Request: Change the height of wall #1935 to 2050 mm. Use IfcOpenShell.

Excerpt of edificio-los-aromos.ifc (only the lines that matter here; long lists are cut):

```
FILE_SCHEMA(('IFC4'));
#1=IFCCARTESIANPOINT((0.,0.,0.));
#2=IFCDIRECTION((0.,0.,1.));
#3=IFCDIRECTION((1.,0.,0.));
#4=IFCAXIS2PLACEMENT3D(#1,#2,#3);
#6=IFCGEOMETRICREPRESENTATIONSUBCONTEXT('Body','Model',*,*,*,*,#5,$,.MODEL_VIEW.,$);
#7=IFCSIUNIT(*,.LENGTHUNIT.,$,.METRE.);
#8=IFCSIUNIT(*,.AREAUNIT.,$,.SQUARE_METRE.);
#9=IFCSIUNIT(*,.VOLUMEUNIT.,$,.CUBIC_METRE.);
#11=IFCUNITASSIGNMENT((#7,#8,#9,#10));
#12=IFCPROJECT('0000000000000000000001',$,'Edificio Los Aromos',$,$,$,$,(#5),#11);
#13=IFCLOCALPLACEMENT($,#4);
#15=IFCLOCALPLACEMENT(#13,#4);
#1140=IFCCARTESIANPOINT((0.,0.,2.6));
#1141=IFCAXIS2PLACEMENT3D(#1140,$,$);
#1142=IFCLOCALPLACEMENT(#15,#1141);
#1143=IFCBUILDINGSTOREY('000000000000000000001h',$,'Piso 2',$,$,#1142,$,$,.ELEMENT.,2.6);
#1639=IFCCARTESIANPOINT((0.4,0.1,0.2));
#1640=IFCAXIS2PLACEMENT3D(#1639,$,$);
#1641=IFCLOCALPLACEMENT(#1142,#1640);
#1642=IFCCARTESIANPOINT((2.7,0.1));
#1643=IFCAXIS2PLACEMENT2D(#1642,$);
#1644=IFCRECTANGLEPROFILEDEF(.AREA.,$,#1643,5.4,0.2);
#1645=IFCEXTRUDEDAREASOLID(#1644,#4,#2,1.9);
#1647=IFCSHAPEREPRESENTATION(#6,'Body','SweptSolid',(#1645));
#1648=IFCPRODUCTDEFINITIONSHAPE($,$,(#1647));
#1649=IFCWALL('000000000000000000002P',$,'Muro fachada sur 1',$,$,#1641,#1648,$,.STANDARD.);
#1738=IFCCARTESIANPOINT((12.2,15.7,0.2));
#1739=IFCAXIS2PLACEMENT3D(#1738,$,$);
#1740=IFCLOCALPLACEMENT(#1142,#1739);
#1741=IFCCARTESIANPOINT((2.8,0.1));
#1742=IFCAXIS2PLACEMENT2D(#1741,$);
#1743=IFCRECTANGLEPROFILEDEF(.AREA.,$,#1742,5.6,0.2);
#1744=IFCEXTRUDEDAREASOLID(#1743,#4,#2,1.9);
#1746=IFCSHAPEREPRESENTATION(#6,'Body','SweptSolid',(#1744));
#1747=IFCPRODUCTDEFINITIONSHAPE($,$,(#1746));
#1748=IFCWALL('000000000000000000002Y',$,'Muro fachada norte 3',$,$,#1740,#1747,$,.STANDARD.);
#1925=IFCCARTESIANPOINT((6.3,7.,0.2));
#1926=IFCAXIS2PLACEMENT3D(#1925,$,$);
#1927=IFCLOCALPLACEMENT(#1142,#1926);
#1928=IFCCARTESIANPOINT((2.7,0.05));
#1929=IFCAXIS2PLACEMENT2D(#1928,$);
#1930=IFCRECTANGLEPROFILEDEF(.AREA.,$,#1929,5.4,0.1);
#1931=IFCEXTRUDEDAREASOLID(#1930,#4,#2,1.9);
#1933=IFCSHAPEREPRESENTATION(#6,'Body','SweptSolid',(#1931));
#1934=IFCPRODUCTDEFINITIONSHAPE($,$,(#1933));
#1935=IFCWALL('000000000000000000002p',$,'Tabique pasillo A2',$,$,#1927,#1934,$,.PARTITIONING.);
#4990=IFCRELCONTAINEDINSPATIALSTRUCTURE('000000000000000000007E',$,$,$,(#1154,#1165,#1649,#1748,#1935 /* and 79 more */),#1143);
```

```python
import ifcopenshell
import ifcopenshell.geom
import ifcopenshell.util.representation
import ifcopenshell.util.shape
import ifcopenshell.util.unit

model = ifcopenshell.open("edificio-los-aromos.ifc")
unit_scale = ifcopenshell.util.unit.calculate_unit_scale(model)
settings = ifcopenshell.geom.settings()


def volume(element):
    """Net volume in cubic metres, openings subtracted."""
    shape = ifcopenshell.geom.create_shape(settings, element)
    return ifcopenshell.util.shape.get_volume(shape.geometry)


wall = model.by_guid("000000000000000000002p")
before = volume(wall)

body = ifcopenshell.util.representation.get_representation(wall, "Model", "Body")
solid = body.Items[0]
old_height = solid.Depth
solid.Depth = 2.05 / unit_scale
after = volume(wall)

print(f"height {old_height:g} -> {solid.Depth:g}, volume {before:.3f} -> {after:.3f} m3")

model.write("edificio-los-aromos_rev.ifc")
```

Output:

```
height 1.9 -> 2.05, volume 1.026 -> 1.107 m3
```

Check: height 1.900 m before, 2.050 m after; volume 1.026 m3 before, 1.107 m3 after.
